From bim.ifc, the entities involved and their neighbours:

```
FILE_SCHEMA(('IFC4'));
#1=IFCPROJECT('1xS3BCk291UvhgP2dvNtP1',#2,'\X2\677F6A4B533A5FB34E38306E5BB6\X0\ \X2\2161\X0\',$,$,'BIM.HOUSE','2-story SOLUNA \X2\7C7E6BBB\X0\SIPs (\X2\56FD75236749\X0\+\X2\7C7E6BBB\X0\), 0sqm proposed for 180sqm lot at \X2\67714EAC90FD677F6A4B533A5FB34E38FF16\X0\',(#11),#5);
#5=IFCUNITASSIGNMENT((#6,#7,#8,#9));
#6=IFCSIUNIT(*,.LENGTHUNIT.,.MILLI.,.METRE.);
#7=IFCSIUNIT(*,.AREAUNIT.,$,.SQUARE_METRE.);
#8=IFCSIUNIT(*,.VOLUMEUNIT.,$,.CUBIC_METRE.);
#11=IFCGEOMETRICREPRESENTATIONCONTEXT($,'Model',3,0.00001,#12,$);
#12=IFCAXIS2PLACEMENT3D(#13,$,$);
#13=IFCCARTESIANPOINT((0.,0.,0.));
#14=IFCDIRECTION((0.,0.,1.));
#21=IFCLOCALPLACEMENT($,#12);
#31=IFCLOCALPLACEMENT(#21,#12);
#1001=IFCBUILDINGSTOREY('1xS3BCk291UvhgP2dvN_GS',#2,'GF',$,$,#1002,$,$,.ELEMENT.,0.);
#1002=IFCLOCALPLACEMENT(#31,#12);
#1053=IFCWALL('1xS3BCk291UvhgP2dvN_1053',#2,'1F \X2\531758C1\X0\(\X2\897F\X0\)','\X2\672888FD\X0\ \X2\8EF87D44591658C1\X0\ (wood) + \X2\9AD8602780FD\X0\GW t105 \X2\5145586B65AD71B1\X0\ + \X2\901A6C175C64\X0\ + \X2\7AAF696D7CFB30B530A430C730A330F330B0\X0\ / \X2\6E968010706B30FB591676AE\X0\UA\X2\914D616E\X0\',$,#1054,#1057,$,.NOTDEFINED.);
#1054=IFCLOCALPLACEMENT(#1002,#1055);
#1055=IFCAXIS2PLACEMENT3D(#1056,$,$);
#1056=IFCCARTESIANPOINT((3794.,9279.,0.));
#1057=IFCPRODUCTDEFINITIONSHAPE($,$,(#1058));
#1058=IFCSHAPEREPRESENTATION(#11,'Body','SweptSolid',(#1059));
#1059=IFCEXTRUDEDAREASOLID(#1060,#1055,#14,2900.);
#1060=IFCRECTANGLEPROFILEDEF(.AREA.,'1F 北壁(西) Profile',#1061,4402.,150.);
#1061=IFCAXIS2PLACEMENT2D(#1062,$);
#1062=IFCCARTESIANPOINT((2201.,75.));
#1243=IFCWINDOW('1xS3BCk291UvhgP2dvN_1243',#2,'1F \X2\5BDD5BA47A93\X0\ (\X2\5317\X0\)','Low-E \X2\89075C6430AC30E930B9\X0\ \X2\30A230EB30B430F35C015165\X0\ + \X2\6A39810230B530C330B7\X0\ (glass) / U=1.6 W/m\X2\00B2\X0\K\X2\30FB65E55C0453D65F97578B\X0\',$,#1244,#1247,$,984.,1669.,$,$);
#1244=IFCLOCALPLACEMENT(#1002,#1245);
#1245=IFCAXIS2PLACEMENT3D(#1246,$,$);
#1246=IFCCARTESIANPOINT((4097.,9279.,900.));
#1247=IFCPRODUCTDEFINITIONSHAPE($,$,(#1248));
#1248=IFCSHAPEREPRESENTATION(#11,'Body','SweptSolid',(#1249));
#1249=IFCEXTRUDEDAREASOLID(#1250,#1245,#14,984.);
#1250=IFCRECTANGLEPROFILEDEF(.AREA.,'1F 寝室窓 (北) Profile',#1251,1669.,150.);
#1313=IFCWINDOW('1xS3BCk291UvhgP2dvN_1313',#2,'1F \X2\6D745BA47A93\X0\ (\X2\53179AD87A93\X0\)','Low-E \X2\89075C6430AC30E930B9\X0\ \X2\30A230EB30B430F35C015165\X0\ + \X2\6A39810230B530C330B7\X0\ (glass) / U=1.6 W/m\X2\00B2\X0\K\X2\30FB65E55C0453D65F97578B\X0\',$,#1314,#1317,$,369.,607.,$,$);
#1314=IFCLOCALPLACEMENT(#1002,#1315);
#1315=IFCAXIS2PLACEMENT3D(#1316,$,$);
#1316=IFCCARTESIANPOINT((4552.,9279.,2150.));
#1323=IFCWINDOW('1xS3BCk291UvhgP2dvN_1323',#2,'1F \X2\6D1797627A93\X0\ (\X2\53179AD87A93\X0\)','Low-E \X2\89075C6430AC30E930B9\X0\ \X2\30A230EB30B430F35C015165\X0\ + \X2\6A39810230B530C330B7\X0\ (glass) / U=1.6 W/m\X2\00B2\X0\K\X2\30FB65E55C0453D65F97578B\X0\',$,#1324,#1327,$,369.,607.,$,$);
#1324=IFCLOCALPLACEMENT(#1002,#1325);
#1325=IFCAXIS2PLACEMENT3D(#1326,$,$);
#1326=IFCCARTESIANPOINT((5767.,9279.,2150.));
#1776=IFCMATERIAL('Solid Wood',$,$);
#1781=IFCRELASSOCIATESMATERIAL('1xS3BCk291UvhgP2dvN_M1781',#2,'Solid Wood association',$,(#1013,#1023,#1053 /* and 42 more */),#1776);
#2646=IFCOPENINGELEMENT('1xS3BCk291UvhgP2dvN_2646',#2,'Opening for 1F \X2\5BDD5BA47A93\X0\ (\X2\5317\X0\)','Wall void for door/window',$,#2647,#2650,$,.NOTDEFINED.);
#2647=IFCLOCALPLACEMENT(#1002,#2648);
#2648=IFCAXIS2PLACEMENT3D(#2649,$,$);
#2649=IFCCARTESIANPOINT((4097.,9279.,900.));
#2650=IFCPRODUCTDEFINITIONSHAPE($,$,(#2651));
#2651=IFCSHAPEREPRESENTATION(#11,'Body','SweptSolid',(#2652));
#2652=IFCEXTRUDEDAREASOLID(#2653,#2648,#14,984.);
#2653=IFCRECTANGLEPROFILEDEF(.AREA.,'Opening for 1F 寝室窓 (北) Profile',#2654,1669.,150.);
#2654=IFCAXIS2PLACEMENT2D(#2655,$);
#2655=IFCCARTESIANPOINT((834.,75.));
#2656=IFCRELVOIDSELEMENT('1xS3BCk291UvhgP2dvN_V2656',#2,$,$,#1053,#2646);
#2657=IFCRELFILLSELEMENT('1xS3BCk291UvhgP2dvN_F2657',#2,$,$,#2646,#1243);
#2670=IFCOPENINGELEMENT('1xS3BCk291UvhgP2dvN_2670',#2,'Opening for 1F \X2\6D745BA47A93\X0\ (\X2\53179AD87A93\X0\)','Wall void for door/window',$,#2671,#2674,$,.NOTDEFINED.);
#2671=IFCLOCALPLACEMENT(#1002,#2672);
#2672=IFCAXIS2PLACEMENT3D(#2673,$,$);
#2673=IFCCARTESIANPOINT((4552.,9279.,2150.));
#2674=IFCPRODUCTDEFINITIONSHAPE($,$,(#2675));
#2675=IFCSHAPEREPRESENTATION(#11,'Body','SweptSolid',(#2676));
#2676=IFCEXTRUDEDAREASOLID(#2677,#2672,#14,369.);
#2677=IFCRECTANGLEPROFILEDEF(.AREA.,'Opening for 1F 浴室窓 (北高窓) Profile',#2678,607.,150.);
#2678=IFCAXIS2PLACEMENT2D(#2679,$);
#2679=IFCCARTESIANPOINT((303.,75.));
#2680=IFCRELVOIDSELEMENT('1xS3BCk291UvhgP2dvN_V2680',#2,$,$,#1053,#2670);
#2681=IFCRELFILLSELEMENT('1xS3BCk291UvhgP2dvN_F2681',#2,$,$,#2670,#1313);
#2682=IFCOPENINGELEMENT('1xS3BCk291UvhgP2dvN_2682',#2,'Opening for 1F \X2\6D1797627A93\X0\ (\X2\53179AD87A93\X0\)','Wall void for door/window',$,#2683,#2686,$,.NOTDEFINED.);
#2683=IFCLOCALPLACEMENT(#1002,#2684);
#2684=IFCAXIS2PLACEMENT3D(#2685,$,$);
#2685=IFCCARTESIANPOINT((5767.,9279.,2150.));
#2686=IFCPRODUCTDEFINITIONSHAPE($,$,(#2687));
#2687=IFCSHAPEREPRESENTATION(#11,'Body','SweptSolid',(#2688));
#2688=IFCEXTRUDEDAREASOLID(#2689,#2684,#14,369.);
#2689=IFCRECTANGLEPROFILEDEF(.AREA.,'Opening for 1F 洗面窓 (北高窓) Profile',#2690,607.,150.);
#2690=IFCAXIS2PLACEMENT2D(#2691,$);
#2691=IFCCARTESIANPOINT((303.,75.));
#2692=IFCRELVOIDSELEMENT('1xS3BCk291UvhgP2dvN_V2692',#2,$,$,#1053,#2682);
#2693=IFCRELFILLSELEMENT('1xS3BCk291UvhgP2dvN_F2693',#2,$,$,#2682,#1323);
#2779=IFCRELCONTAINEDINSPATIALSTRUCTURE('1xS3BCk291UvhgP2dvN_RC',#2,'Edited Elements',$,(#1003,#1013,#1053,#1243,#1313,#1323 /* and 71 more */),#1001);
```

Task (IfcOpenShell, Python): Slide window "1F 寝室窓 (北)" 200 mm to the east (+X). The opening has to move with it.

```python
import ifcopenshell
import ifcopenshell.api.geometry
import ifcopenshell.util.placement
import ifcopenshell.util.unit

model = ifcopenshell.open("bim.ifc")
unit_scale = ifcopenshell.util.unit.calculate_unit_scale(model)

window = model.by_guid("1xS3BCk291UvhgP2dvN_1243")
opening = window.FillsVoids[0].RelatingOpeningElement
wall = opening.VoidsElements[0].RelatingBuildingElement

wall_matrix = ifcopenshell.util.placement.get_local_placement(wall.ObjectPlacement)
shift = wall_matrix[:3, 0] * 0.2 / unit_scale
before = ifcopenshell.util.placement.get_local_placement(window.ObjectPlacement)[:3, 3].copy()

# The window is not placed relative to its opening, so move both.
for product in (opening, window):
    matrix = ifcopenshell.util.placement.get_local_placement(product.ObjectPlacement)
    matrix[:3, 3] += shift
    ifcopenshell.api.geometry.edit_object_placement(model, product=product, matrix=matrix, is_si=False)

after = ifcopenshell.util.placement.get_local_placement(window.ObjectPlacement)[:3, 3]
print("window moved by", (after - before).round(3) + 0.0)

model.write("bim_edited.ifc")
```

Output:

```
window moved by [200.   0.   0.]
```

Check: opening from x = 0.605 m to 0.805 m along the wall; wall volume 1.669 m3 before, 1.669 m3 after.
